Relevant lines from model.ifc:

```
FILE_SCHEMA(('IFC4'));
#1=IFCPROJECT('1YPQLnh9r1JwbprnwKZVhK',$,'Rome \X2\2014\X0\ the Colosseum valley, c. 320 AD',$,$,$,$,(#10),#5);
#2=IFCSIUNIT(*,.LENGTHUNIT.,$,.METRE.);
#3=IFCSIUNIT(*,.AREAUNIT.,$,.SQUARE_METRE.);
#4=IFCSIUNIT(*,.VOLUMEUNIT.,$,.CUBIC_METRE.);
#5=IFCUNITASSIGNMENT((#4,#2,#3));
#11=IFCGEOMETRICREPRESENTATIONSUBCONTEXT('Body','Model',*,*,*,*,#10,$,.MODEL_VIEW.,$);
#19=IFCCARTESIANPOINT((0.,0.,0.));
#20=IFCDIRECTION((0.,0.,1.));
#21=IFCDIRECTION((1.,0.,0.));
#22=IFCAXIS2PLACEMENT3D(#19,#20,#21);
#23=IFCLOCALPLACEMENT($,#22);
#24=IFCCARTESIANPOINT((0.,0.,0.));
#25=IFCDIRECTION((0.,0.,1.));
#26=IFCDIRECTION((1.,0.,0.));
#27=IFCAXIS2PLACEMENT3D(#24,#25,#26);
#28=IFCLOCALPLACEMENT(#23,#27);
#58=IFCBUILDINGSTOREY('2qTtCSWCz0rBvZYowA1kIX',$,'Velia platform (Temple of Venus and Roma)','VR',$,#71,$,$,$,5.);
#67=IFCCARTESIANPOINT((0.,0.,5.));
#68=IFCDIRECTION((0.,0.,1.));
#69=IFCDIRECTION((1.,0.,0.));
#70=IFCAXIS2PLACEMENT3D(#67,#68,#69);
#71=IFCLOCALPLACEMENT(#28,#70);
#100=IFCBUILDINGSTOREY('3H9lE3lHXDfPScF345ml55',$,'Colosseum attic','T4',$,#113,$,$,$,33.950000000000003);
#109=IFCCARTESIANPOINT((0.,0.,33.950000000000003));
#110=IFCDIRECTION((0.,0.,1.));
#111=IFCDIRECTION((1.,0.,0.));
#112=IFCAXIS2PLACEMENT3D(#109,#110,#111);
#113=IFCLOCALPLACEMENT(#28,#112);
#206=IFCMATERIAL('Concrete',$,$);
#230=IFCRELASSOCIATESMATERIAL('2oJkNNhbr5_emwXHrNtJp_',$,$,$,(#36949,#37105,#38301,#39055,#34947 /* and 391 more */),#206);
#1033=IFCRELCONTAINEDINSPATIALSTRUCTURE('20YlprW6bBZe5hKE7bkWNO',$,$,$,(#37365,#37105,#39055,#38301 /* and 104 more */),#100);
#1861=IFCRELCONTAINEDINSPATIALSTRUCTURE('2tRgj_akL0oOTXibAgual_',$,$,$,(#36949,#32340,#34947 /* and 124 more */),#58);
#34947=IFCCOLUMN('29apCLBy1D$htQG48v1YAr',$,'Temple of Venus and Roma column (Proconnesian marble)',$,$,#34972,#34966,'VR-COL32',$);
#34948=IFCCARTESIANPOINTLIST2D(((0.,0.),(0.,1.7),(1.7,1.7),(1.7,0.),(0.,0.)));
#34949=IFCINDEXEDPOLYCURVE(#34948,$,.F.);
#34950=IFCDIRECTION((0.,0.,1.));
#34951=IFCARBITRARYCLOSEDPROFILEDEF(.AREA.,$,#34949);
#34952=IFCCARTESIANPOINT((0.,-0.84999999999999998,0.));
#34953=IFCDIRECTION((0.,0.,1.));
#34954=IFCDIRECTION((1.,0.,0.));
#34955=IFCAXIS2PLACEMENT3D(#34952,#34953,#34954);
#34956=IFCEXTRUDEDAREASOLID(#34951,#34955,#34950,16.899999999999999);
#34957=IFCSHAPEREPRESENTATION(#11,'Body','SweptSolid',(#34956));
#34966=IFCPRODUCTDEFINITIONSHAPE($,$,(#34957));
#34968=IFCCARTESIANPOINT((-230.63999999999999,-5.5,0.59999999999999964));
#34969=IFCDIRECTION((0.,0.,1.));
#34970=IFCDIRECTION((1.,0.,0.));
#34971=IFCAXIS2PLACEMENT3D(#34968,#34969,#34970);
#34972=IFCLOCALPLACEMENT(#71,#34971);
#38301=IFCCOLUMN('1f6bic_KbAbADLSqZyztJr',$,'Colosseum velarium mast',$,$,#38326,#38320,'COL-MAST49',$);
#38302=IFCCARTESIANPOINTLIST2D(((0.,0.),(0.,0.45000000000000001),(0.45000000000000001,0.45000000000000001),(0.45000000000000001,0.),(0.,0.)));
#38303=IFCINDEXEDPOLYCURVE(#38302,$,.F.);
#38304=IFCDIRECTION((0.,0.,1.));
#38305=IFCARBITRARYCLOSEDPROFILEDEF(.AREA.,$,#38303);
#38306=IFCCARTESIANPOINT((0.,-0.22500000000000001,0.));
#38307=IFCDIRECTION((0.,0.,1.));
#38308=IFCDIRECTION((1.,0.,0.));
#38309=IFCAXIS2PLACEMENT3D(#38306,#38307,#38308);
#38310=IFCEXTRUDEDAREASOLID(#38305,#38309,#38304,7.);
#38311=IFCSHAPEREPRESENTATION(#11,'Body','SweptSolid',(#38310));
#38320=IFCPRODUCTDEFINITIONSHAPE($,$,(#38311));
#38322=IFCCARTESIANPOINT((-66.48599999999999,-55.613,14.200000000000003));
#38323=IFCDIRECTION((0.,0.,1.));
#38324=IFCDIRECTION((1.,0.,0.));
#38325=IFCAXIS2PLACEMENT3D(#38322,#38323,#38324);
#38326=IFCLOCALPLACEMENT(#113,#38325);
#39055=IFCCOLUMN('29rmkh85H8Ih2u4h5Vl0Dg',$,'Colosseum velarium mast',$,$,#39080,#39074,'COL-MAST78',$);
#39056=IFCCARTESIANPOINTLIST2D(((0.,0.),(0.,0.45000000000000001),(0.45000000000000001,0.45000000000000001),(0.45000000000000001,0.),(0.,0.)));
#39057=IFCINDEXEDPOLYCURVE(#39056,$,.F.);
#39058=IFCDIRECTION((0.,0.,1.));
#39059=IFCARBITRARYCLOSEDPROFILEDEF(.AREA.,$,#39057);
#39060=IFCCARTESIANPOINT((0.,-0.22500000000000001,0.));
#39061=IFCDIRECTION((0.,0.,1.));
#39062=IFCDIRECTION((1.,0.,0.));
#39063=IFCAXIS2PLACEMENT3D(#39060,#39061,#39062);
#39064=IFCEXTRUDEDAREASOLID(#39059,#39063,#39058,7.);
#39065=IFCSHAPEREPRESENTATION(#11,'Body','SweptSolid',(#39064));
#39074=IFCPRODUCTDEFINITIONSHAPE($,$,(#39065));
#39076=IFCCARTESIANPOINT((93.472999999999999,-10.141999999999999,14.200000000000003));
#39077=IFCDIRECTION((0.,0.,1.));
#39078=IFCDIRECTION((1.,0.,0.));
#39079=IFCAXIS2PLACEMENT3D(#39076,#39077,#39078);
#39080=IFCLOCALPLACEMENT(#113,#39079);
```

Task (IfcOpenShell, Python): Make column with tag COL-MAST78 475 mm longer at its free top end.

```python
import ifcopenshell
import ifcopenshell.util.representation

model = ifcopenshell.open("model.ifc")

member = model.by_id(39055)
change = 0.475

# The extrusion runs towards the end named, so only its depth changes.
body = ifcopenshell.util.representation.get_representation(member, "Model", "Body")
solid = body.Items[0]
old_length = solid.Depth
solid.Depth += change

print(f"length {old_length:g} -> {solid.Depth:g}")

model.write("model_updated.ifc")
```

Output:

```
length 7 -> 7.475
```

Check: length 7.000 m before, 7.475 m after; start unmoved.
